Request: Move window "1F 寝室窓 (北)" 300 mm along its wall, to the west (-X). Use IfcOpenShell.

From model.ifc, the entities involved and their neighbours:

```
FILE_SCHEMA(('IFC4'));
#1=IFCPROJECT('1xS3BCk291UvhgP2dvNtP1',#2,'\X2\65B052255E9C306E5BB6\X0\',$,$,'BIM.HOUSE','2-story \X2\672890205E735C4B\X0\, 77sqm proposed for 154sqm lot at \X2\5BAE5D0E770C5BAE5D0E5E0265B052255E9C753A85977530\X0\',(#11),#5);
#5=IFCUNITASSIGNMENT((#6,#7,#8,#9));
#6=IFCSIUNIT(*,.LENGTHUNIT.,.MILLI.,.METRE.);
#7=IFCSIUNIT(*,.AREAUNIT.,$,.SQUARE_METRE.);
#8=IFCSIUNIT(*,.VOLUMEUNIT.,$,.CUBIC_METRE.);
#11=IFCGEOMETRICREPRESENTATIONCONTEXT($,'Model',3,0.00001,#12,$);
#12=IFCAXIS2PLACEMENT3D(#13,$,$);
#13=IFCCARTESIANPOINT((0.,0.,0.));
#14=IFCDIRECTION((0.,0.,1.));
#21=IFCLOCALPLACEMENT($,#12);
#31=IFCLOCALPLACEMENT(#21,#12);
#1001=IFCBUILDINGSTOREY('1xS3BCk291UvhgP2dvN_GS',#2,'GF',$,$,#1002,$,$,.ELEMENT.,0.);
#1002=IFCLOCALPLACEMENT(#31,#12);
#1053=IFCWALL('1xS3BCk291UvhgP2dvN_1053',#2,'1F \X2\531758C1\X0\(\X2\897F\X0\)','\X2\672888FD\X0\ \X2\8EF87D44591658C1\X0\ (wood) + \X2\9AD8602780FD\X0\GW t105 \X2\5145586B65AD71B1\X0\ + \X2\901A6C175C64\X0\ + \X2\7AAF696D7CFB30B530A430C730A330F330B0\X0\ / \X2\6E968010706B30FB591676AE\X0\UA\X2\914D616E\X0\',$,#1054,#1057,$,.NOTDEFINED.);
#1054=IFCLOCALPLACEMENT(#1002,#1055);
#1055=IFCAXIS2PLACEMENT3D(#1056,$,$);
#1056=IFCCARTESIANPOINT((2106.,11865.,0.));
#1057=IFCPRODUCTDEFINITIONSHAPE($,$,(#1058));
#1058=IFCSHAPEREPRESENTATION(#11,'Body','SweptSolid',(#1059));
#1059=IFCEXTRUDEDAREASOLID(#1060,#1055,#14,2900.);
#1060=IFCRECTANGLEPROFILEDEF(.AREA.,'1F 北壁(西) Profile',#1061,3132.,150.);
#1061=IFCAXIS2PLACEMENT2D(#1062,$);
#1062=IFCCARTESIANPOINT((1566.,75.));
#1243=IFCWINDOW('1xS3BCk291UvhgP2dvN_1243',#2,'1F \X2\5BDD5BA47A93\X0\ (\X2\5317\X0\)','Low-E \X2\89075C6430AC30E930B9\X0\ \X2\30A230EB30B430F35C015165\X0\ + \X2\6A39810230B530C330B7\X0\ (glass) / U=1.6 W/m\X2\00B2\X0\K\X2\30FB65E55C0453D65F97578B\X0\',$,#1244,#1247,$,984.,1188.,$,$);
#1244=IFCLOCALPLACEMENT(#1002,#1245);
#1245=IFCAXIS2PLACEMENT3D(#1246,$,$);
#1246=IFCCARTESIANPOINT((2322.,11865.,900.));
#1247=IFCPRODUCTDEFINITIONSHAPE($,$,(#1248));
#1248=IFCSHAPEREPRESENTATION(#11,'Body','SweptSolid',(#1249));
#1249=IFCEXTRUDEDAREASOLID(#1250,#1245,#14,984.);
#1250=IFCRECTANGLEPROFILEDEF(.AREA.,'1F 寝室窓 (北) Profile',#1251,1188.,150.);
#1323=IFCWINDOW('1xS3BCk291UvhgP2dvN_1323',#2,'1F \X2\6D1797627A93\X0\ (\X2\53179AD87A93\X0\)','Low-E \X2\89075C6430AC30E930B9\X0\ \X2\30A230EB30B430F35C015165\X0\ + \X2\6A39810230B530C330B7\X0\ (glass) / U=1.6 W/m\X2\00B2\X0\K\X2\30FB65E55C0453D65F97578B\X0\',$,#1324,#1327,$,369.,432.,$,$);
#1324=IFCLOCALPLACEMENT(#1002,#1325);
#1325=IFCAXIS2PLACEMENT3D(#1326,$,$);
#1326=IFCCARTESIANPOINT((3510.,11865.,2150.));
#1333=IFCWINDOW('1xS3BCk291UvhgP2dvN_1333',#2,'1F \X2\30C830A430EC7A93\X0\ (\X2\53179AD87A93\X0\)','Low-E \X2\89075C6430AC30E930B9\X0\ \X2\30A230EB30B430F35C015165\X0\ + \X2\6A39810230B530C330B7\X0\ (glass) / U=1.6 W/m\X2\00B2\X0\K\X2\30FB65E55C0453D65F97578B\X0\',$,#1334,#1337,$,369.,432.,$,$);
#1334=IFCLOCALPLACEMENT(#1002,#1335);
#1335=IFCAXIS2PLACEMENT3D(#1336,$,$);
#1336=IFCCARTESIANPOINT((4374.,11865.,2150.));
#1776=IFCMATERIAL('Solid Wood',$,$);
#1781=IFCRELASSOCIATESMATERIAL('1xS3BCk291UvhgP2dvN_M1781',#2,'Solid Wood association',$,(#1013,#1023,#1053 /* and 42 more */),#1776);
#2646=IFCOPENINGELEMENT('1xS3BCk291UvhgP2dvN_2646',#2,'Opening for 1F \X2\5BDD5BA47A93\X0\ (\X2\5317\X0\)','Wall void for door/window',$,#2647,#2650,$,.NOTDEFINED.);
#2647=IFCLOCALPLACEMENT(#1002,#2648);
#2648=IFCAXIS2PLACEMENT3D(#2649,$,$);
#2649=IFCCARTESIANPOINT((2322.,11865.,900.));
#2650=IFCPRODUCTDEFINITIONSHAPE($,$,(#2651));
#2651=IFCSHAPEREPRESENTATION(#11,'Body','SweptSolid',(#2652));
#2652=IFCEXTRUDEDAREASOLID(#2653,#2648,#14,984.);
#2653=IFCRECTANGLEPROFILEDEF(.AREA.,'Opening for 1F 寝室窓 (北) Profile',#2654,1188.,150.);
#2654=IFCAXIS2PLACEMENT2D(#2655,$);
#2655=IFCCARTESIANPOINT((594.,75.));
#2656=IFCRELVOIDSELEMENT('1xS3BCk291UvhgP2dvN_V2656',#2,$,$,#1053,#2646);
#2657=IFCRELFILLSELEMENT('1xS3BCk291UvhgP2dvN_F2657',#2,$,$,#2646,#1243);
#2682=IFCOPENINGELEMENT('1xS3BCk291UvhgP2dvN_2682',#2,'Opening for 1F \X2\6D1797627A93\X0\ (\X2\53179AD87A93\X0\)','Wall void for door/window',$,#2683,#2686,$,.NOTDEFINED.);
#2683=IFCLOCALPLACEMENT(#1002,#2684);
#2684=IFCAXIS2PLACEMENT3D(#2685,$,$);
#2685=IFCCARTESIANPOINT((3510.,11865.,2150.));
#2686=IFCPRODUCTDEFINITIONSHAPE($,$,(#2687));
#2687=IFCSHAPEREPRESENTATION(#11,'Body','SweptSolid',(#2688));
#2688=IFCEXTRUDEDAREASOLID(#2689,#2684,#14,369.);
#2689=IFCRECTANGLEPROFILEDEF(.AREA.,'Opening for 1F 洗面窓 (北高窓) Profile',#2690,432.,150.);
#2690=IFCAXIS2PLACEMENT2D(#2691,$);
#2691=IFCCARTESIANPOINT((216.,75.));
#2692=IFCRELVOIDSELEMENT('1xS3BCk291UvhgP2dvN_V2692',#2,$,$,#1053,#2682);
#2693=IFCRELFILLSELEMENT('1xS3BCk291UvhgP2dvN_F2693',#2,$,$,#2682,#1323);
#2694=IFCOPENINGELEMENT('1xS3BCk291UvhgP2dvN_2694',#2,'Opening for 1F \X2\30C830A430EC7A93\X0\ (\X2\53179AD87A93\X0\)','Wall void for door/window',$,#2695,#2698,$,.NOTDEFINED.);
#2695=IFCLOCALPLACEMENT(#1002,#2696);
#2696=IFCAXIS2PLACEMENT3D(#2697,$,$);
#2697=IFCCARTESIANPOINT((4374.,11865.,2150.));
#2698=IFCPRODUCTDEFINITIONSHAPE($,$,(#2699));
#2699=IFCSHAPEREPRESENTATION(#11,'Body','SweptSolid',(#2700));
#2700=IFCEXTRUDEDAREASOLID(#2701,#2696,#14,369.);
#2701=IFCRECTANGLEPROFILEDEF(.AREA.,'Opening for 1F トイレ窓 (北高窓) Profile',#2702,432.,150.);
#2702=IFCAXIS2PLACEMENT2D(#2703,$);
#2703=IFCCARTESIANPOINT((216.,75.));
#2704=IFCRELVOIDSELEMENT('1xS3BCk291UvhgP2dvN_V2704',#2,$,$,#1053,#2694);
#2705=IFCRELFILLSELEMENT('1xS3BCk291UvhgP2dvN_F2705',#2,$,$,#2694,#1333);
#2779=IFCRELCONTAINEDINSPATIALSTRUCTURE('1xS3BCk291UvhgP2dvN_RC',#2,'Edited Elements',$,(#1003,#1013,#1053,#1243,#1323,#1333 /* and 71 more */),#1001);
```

```python
import ifcopenshell
import ifcopenshell.api.geometry
import ifcopenshell.util.placement
import ifcopenshell.util.unit

model = ifcopenshell.open("model.ifc")
unit_scale = ifcopenshell.util.unit.calculate_unit_scale(model)

window = model.by_id(1243)
opening = window.FillsVoids[0].RelatingOpeningElement
wall = opening.VoidsElements[0].RelatingBuildingElement

wall_matrix = ifcopenshell.util.placement.get_local_placement(wall.ObjectPlacement)
shift = wall_matrix[:3, 0] * -0.3 / unit_scale
before = ifcopenshell.util.placement.get_local_placement(window.ObjectPlacement)[:3, 3].copy()

# The window is not placed relative to its opening, so move both.
for product in (opening, window):
    matrix = ifcopenshell.util.placement.get_local_placement(product.ObjectPlacement)
    matrix[:3, 3] += shift
    ifcopenshell.api.geometry.edit_object_placement(model, product=product, matrix=matrix, is_si=False)

after = ifcopenshell.util.placement.get_local_placement(window.ObjectPlacement)[:3, 3]
print("window moved by", (after - before).round(3) + 0.0)

model.write("model-out.ifc")
```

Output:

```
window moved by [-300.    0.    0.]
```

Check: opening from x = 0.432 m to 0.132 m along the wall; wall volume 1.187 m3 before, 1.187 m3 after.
